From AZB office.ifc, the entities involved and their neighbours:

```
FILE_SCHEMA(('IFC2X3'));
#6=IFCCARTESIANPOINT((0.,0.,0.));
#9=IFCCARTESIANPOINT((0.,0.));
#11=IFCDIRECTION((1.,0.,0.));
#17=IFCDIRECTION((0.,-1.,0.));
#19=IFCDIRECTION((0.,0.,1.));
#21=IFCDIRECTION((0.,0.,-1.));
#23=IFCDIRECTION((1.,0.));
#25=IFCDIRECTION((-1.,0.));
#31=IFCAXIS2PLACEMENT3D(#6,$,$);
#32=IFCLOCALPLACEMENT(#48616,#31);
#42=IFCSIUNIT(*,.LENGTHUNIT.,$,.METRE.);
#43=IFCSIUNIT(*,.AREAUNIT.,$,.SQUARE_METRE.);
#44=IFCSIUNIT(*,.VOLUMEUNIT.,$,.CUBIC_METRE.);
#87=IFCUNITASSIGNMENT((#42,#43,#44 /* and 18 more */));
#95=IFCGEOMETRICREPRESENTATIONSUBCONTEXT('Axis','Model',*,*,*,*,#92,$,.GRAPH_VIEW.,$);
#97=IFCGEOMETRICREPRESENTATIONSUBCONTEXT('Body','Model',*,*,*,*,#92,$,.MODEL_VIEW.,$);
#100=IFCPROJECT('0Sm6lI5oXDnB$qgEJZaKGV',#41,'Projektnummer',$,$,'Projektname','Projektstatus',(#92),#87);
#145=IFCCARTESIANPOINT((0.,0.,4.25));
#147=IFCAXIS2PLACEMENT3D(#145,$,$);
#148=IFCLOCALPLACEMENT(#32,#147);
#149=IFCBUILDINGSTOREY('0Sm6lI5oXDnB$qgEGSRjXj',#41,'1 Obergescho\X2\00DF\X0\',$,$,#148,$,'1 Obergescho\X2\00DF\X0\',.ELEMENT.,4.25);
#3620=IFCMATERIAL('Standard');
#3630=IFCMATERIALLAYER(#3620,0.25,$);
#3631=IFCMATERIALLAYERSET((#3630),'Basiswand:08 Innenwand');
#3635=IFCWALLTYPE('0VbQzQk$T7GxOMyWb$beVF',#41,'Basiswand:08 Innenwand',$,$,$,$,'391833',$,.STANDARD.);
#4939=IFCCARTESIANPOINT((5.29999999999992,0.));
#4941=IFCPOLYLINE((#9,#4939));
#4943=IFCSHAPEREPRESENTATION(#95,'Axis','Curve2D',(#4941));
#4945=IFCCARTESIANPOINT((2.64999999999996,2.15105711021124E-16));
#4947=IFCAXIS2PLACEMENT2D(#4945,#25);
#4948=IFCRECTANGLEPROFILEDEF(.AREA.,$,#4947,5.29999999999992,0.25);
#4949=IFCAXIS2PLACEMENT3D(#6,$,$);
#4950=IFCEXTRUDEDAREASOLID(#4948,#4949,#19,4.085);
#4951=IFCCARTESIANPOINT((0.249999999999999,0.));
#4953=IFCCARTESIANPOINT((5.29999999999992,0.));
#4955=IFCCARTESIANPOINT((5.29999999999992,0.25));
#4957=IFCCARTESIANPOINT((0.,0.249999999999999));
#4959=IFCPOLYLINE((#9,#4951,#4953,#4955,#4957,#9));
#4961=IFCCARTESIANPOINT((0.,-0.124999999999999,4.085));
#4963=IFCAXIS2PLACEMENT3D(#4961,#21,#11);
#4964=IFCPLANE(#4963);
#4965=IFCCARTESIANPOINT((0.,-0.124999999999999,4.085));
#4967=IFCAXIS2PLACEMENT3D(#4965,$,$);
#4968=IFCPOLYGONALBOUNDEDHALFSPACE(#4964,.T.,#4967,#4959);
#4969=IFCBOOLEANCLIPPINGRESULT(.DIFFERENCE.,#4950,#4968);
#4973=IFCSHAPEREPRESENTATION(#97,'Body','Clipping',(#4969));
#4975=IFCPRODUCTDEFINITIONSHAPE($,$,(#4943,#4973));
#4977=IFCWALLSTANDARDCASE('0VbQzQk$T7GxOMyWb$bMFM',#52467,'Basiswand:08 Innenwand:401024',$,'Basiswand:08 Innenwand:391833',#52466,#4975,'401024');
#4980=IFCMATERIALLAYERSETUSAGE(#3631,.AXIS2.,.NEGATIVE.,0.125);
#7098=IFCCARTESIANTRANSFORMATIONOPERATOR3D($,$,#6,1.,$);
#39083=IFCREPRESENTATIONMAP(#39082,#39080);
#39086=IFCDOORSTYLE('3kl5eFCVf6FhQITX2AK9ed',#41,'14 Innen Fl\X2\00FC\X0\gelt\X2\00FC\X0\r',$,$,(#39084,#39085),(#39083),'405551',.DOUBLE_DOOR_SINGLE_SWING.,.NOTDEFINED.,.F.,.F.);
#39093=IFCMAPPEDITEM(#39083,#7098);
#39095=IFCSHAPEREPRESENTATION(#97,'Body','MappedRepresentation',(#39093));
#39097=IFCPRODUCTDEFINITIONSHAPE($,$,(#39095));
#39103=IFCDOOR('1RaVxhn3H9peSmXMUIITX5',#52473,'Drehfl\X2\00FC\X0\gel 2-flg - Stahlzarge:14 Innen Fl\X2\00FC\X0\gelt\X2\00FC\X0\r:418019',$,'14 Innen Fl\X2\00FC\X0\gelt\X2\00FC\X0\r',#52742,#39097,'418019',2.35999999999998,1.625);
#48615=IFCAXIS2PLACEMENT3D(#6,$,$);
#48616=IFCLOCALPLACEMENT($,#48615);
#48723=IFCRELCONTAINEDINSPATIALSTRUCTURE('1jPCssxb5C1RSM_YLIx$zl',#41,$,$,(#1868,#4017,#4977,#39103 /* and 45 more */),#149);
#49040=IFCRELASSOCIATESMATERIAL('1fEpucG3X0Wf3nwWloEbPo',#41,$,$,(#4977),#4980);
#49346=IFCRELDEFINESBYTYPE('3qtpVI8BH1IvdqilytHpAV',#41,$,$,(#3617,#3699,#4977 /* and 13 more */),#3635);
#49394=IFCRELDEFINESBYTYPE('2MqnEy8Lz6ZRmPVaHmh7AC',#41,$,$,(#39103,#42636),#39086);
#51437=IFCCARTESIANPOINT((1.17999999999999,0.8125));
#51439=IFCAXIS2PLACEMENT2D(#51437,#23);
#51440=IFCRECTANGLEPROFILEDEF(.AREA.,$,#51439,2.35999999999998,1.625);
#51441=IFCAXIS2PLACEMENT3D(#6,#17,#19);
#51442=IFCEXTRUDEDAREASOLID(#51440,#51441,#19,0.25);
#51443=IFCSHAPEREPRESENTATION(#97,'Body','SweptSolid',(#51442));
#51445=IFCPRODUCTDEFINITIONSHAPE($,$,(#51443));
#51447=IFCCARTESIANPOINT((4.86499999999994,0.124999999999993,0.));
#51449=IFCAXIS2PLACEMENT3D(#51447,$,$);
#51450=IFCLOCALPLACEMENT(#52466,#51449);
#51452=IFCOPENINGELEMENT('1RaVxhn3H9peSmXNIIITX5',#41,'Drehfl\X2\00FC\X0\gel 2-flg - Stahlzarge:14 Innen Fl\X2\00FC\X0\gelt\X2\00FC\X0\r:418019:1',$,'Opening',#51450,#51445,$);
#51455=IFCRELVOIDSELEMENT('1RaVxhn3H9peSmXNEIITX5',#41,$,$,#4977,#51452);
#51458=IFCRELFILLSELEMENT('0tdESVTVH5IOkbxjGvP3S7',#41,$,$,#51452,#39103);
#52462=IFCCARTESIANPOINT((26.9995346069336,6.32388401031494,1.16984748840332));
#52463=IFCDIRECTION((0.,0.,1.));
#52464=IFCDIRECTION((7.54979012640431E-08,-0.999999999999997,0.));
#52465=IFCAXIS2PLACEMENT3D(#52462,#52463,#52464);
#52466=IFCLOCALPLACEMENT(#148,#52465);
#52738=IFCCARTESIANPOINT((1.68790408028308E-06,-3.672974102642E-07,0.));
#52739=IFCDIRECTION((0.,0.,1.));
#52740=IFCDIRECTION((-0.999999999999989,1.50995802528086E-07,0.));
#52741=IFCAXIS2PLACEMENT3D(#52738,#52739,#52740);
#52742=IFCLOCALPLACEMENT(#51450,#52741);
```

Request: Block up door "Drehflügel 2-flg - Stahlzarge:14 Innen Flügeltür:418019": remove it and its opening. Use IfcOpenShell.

```python
import ifcopenshell
import ifcopenshell.api.feature
import ifcopenshell.api.root
import ifcopenshell.geom
import ifcopenshell.util.shape

model = ifcopenshell.open("AZB office.ifc")
settings = ifcopenshell.geom.settings()


def volume(element):
    """Net volume in cubic metres, openings subtracted."""
    shape = ifcopenshell.geom.create_shape(settings, element)
    return ifcopenshell.util.shape.get_volume(shape.geometry)


door = model.by_id(39103)
opening = door.FillsVoids[0].RelatingOpeningElement
wall = opening.VoidsElements[0].RelatingBuildingElement
before = volume(wall)

ifcopenshell.api.root.remove_product(model, product=door)
ifcopenshell.api.feature.remove_feature(model, feature=opening)

after = volume(wall)

print(f"wall volume {before:.3f} -> {after:.3f} m3")

model.write("AZB office_v2.ifc")
```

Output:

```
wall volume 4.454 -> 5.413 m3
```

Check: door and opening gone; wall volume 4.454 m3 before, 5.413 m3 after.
